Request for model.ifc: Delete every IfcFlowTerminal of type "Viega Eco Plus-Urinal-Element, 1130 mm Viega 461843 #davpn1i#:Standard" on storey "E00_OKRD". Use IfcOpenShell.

First a look at what the model holds.

```python
import ifcopenshell
import ifcopenshell.util.element

model = ifcopenshell.open("model.ifc")
print(model.schema)
storey = next(s for s in model.by_type("IfcBuildingStorey") if s.Name == "E00_OKRD")
terminals = [e for e in ifcopenshell.util.element.get_decomposition(storey) if e.is_a("IfcFlowTerminal")]
seen = {}
for e in terminals:
    element_type = ifcopenshell.util.element.get_type(e)
    name = element_type.Name if element_type not in (None, e) else None
    seen[name] = seen.get(name, 0) + 1
for name, count in sorted(seen.items(), key=str):
    print(count, "x", name)
```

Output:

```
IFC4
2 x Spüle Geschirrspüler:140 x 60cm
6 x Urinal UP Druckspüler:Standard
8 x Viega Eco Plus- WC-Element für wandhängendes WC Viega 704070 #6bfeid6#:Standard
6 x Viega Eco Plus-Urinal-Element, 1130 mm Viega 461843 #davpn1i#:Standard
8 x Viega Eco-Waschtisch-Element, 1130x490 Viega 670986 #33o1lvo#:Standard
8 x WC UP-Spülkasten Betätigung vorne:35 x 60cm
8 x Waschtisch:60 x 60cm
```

```python
import ifcopenshell
import ifcopenshell.api.root
import ifcopenshell.util.element

model = ifcopenshell.open("model.ifc")

storey = next(s for s in model.by_type("IfcBuildingStorey") if s.Name == "E00_OKRD")
terminals = [e for e in ifcopenshell.util.element.get_decomposition(storey) if e.is_a("IfcFlowTerminal")]
targets = [e for e in terminals if (t := ifcopenshell.util.element.get_type(e)) not in (None, e) and t.Name == "Viega Eco Plus-Urinal-Element, 1130 mm Viega 461843 #davpn1i#:Standard"]

for e in targets:
    ifcopenshell.api.root.remove_product(model, product=e)
print(len(targets), "removed")

model.write("model_v2.ifc")
```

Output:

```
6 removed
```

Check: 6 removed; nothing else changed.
